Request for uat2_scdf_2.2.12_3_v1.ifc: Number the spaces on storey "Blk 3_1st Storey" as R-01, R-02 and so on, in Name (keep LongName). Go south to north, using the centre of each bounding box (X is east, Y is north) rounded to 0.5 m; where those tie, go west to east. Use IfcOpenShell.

First a look at what the model holds.

```python
import ifcopenshell
import ifcopenshell.util.element
import ifcopenshell.util.placement

model = ifcopenshell.open("uat2_scdf_2.2.12_3_v1.ifc")
print(model.schema)
storey = next(s for s in model.by_type("IfcBuildingStorey") if s.Name == "Blk 3_1st Storey")
spaces = [e for e in ifcopenshell.util.element.get_decomposition(storey) if e.is_a("IfcSpace")]
for e in sorted(spaces, key=lambda e: e.id()):
    origin = ifcopenshell.util.placement.get_local_placement(e.ObjectPlacement)[:3, 3]
    print(e.id(), e.Name, e.LongName, origin.round(2) + 0.0, sep=" | ")
```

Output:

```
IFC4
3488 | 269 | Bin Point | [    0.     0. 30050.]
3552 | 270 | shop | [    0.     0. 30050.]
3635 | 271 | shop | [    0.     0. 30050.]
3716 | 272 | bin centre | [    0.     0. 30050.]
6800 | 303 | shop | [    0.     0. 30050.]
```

```python
import ifcopenshell
import ifcopenshell.geom
import ifcopenshell.util.element
import ifcopenshell.util.shape

model = ifcopenshell.open("uat2_scdf_2.2.12_3_v1.ifc")
settings = ifcopenshell.geom.settings()
settings.set("use-world-coords", True)


def centre(element):
    shape = ifcopenshell.geom.create_shape(settings, element)
    return ifcopenshell.util.shape.get_bbox_centroid(shape.geometry)


storey = next(s for s in model.by_type("IfcBuildingStorey") if s.Name == "Blk 3_1st Storey")
spaces = [e for e in ifcopenshell.util.element.get_decomposition(storey) if e.is_a("IfcSpace")]

# Insertion points can sit at a corner or the storey origin, so sort by the geometry (in metres).
centres = {e: centre(e) for e in spaces}
spaces.sort(key=lambda e: (round(centres[e][1] / 0.5), centres[e][0]))

for i, e in enumerate(spaces, start=1):
    number = f"R-{i:02d}"
    e.Name = number
    print(e.id(), number)

model.write("uat2_scdf_2.2.12_3_v1_edited.ifc")
```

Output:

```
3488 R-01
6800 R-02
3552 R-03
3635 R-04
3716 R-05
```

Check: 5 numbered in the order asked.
